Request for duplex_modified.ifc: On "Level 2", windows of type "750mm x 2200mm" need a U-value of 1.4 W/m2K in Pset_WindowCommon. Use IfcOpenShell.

First a look at what the model holds.

```python
import ifcopenshell
import ifcopenshell.util.element

model = ifcopenshell.open("duplex_modified.ifc")
print(model.schema)
storey = next(s for s in model.by_type("IfcBuildingStorey") if s.Name == "Level 2")
windows = [e for e in ifcopenshell.util.element.get_decomposition(storey) if e.is_a("IfcWindow")]
seen = {}
for e in windows:
    element_type = ifcopenshell.util.element.get_type(e)
    key = (element_type.Name if element_type != e and element_type else None, ifcopenshell.util.element.get_pset(e, "Pset_WindowCommon", "ThermalTransmittance"))
    seen[key] = seen.get(key, 0) + 1
for (name, value), count in sorted(seen.items(), key=str):
    print(count, "x", name, "|", value)
```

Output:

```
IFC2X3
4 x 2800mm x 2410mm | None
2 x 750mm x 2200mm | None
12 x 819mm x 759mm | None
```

```python
import ifcopenshell
import ifcopenshell.api.pset
import ifcopenshell.util.element

model = ifcopenshell.open("duplex_modified.ifc")

storey = next(s for s in model.by_type("IfcBuildingStorey") if s.Name == "Level 2")
windows = [e for e in ifcopenshell.util.element.get_decomposition(storey) if e.is_a("IfcWindow")]

count = 0
for e in windows:
    element_type = ifcopenshell.util.element.get_type(e)
    if element_type in (None, e) or element_type.Name != "750mm x 2200mm":
        continue
    # add_pset returns the element's existing set when there is one.
    pset = ifcopenshell.api.pset.add_pset(model, product=e, name="Pset_WindowCommon")
    ifcopenshell.api.pset.edit_pset(model, pset=pset, properties={"ThermalTransmittance": 1.4})
    count += 1

print(count, "windows updated")

model.write("duplex_modified_updated.ifc")
```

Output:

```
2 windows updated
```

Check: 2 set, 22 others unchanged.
